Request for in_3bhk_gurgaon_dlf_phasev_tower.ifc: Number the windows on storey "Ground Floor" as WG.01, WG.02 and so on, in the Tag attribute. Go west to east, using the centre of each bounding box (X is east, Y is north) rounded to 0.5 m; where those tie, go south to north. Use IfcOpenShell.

First a look at what the model holds.

```python
import ifcopenshell
import ifcopenshell.util.element
import ifcopenshell.util.placement

model = ifcopenshell.open("in_3bhk_gurgaon_dlf_phasev_tower.ifc")
print(model.schema)
storey = next(s for s in model.by_type("IfcBuildingStorey") if s.Name == "Ground Floor")
windows = [e for e in ifcopenshell.util.element.get_decomposition(storey) if e.is_a("IfcWindow")]
for e in sorted(windows, key=lambda e: e.id()):
    origin = ifcopenshell.util.placement.get_local_placement(e.ObjectPlacement)[:3, 3]
    print(e.id(), e.Tag, e.Name, origin.round(2) + 0.0, sep=" | ")
```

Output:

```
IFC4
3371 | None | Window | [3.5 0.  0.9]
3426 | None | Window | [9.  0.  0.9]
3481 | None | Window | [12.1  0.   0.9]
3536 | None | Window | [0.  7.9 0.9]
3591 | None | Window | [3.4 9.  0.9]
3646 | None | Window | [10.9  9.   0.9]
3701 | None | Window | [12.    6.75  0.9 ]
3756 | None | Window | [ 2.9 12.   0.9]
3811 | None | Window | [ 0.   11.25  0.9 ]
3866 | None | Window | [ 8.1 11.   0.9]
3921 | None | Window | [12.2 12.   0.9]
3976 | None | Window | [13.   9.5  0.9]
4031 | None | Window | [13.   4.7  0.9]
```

```python
import ifcopenshell
import ifcopenshell.geom
import ifcopenshell.util.element
import ifcopenshell.util.shape

model = ifcopenshell.open("in_3bhk_gurgaon_dlf_phasev_tower.ifc")
settings = ifcopenshell.geom.settings()
settings.set("use-world-coords", True)


def centre(element):
    shape = ifcopenshell.geom.create_shape(settings, element)
    return ifcopenshell.util.shape.get_bbox_centroid(shape.geometry)


storey = next(s for s in model.by_type("IfcBuildingStorey") if s.Name == "Ground Floor")
windows = [e for e in ifcopenshell.util.element.get_decomposition(storey) if e.is_a("IfcWindow")]

# Insertion points can sit at a corner or the storey origin, so sort by the geometry (in metres).
centres = {e: centre(e) for e in windows}
windows.sort(key=lambda e: (round(centres[e][0] / 0.5), centres[e][1]))

for i, e in enumerate(windows, start=1):
    number = f"WG.{i:02d}"
    e.Tag = number
    print(e.id(), number)

model.write("in_3bhk_gurgaon_dlf_phasev_tower_edited.ifc")
```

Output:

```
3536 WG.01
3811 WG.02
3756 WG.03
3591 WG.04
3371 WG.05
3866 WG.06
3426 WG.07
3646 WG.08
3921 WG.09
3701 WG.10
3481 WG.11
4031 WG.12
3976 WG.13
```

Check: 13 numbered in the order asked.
